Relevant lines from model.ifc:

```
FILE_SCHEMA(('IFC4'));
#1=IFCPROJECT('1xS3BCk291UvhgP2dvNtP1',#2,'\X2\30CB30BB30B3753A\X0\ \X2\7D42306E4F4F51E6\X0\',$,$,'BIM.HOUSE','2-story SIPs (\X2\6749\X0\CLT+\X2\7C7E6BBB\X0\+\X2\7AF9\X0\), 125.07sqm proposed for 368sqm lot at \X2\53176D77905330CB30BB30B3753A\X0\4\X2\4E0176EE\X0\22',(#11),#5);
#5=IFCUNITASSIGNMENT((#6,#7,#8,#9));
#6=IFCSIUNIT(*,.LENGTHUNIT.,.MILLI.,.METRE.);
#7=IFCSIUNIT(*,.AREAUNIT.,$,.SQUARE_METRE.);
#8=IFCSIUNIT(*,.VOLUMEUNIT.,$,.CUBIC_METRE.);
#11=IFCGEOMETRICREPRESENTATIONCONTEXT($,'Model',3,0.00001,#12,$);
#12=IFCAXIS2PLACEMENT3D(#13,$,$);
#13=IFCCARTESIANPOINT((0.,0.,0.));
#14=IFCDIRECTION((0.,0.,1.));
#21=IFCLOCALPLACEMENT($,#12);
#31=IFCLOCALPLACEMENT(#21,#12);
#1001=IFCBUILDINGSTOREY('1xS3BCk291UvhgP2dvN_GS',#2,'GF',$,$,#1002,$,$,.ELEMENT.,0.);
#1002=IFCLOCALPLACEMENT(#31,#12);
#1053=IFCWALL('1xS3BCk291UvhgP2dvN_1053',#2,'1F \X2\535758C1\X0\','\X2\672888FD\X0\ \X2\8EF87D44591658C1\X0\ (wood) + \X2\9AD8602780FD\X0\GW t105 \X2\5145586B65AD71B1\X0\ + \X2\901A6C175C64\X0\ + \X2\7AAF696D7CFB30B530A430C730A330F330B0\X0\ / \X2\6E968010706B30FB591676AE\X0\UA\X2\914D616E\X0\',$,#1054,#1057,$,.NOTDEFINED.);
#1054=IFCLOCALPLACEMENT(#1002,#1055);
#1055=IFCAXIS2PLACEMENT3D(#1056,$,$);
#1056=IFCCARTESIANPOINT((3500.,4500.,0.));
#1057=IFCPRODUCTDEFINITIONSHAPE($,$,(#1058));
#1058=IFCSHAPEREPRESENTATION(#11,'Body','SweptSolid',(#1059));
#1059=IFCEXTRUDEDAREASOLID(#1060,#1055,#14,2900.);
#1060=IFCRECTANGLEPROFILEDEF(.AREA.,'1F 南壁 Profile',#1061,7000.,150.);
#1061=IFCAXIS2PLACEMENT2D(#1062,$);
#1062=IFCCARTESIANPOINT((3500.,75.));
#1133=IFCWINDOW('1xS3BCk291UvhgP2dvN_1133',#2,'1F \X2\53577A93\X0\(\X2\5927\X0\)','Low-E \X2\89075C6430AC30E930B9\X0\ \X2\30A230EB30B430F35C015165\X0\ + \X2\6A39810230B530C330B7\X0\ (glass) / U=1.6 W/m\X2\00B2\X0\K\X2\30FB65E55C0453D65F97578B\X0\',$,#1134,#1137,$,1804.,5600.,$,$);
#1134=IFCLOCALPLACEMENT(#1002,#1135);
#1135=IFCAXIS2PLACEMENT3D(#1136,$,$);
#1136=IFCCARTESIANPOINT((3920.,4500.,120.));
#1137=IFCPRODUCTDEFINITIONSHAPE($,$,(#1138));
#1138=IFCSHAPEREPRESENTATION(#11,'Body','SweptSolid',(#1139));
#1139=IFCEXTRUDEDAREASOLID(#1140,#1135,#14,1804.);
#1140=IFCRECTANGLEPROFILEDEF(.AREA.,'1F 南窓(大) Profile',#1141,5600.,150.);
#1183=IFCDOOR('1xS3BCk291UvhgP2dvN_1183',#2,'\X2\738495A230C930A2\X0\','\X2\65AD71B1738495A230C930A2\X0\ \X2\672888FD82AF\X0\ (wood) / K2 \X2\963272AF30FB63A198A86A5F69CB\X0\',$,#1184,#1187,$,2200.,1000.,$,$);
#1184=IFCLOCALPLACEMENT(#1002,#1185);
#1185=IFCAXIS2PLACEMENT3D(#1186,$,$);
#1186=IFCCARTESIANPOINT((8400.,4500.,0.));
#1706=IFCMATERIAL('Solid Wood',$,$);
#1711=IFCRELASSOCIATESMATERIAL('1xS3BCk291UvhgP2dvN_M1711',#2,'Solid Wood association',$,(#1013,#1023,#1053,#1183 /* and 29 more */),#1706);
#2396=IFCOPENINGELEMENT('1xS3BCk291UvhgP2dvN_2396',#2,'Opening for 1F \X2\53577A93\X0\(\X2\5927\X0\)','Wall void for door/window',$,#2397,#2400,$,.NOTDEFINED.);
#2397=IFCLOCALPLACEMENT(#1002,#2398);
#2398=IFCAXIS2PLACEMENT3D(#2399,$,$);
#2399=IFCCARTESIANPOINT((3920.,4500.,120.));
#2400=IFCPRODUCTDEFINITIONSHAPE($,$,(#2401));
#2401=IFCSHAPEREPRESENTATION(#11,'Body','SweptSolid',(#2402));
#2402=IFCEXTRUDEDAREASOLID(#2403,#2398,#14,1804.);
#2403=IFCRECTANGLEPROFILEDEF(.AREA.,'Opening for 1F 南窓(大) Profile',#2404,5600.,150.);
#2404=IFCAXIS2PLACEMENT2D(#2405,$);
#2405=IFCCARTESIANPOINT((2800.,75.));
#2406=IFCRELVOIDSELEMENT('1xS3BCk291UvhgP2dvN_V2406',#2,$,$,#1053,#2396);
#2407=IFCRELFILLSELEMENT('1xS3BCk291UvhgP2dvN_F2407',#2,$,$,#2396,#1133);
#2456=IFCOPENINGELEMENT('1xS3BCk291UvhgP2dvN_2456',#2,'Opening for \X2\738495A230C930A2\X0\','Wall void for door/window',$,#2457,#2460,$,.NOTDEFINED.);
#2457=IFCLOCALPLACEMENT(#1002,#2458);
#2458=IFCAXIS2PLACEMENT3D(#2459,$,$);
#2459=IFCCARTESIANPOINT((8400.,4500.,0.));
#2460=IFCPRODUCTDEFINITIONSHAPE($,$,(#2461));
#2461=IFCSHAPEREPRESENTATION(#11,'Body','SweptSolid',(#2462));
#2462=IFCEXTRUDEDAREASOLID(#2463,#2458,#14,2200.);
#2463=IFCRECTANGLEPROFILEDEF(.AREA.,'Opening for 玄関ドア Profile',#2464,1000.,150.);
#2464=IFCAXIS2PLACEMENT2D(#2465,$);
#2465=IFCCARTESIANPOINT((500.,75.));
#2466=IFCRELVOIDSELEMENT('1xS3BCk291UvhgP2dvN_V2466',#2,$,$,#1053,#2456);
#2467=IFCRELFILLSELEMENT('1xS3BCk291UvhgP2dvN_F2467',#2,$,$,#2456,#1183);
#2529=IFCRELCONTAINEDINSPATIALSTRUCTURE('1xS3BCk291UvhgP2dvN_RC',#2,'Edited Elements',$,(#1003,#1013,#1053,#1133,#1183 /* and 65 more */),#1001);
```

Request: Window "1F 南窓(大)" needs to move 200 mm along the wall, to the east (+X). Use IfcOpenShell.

```python
import ifcopenshell
import ifcopenshell.api.geometry
import ifcopenshell.util.placement
import ifcopenshell.util.unit

model = ifcopenshell.open("model.ifc")
unit_scale = ifcopenshell.util.unit.calculate_unit_scale(model)

window = model.by_guid("1xS3BCk291UvhgP2dvN_1133")
opening = window.FillsVoids[0].RelatingOpeningElement
wall = opening.VoidsElements[0].RelatingBuildingElement

wall_matrix = ifcopenshell.util.placement.get_local_placement(wall.ObjectPlacement)
shift = wall_matrix[:3, 0] * 0.2 / unit_scale
before = ifcopenshell.util.placement.get_local_placement(window.ObjectPlacement)[:3, 3].copy()

# The window is not placed relative to its opening, so move both.
for product in (opening, window):
    matrix = ifcopenshell.util.placement.get_local_placement(product.ObjectPlacement)
    matrix[:3, 3] += shift
    ifcopenshell.api.geometry.edit_object_placement(model, product=product, matrix=matrix, is_si=False)

after = ifcopenshell.util.placement.get_local_placement(window.ObjectPlacement)[:3, 3]
print("window moved by", (after - before).round(3) + 0.0)

model.write("model_v2.ifc")
```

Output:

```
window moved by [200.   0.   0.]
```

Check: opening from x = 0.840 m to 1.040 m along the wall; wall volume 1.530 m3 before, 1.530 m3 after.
